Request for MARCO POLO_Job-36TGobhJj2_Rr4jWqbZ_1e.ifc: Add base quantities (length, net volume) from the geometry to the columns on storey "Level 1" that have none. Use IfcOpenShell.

First a look at what the model holds.

```python
import ifcopenshell
import ifcopenshell.util.element
import ifcopenshell.util.unit

model = ifcopenshell.open("MARCO POLO_Job-36TGobhJj2_Rr4jWqbZ_1e.ifc")
print(model.schema)
for unit_type in ("LENGTHUNIT", "AREAUNIT", "VOLUMEUNIT"):
    print(unit_type, ifcopenshell.util.unit.calculate_unit_scale(model, unit_type))
storey = next(s for s in model.by_type("IfcBuildingStorey") if s.Name == "Level 1")
columns = [e for e in ifcopenshell.util.element.get_decomposition(storey) if e.is_a("IfcColumn")]
for e in sorted(columns, key=lambda e: e.id()):
    print(e.id(), e.is_a(), e.Name, list(ifcopenshell.util.element.get_psets(e, qtos_only=True)), sep=" | ")
```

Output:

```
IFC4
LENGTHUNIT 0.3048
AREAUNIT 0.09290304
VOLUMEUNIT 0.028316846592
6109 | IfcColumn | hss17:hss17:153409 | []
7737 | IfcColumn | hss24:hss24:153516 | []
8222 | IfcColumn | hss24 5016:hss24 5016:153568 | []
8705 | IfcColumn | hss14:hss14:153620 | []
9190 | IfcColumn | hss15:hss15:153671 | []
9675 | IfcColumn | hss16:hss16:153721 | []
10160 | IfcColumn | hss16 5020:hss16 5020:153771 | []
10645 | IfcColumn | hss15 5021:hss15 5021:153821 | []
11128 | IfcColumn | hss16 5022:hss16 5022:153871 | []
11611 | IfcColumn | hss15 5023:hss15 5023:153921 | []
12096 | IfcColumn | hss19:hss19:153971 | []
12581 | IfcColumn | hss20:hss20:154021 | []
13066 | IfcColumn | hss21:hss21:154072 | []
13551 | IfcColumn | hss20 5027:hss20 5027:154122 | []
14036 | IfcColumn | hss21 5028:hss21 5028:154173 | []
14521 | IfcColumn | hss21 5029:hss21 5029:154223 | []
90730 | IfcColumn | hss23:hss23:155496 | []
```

```python
import ifcopenshell
import ifcopenshell.api.pset
import ifcopenshell.geom
import ifcopenshell.util.element
import ifcopenshell.util.shape
import ifcopenshell.util.unit

model = ifcopenshell.open("MARCO POLO_Job-36TGobhJj2_Rr4jWqbZ_1e.ifc")
unit_scale = ifcopenshell.util.unit.calculate_unit_scale(model)
volume_scale = ifcopenshell.util.unit.calculate_unit_scale(model, "VOLUMEUNIT")
settings = ifcopenshell.geom.settings()

storey = next(s for s in model.by_type("IfcBuildingStorey") if s.Name == "Level 1")
columns = [e for e in ifcopenshell.util.element.get_decomposition(storey) if e.is_a("IfcColumn")]

for e in sorted(columns, key=lambda e: e.id()):
    if ifcopenshell.util.element.get_psets(e, qtos_only=True, should_inherit=False):
        continue
    # Geometry comes back in metres, in the element's own axes.
    shape = ifcopenshell.geom.create_shape(settings, e)
    values = {
        "Length": ifcopenshell.util.shape.get_z(shape.geometry) / unit_scale,
        "NetVolume": ifcopenshell.util.shape.get_volume(shape.geometry) / volume_scale,
    }
    qto = ifcopenshell.api.pset.add_qto(model, product=e, name="Qto_ColumnBaseQuantities")
    ifcopenshell.api.pset.edit_qto(model, qto=qto, properties=values)
    print(e.id(), {k: round(v, 3) for k, v in values.items()})

model.write("MARCO POLO_Job-36TGobhJj2_Rr4jWqbZ_1e_v2.ifc")
```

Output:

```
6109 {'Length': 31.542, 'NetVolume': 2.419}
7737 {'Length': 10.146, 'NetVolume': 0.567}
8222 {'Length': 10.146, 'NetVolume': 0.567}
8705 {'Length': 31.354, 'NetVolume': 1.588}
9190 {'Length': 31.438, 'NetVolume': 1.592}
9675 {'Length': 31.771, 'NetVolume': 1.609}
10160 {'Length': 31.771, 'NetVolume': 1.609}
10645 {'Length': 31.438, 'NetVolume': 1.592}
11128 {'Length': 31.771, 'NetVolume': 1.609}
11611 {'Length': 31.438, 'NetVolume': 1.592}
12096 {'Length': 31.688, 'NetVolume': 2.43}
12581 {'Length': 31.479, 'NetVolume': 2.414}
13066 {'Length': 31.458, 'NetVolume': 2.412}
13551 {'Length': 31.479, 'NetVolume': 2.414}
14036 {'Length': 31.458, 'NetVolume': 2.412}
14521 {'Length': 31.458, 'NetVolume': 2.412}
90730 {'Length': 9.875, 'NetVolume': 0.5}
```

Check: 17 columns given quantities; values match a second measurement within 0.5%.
